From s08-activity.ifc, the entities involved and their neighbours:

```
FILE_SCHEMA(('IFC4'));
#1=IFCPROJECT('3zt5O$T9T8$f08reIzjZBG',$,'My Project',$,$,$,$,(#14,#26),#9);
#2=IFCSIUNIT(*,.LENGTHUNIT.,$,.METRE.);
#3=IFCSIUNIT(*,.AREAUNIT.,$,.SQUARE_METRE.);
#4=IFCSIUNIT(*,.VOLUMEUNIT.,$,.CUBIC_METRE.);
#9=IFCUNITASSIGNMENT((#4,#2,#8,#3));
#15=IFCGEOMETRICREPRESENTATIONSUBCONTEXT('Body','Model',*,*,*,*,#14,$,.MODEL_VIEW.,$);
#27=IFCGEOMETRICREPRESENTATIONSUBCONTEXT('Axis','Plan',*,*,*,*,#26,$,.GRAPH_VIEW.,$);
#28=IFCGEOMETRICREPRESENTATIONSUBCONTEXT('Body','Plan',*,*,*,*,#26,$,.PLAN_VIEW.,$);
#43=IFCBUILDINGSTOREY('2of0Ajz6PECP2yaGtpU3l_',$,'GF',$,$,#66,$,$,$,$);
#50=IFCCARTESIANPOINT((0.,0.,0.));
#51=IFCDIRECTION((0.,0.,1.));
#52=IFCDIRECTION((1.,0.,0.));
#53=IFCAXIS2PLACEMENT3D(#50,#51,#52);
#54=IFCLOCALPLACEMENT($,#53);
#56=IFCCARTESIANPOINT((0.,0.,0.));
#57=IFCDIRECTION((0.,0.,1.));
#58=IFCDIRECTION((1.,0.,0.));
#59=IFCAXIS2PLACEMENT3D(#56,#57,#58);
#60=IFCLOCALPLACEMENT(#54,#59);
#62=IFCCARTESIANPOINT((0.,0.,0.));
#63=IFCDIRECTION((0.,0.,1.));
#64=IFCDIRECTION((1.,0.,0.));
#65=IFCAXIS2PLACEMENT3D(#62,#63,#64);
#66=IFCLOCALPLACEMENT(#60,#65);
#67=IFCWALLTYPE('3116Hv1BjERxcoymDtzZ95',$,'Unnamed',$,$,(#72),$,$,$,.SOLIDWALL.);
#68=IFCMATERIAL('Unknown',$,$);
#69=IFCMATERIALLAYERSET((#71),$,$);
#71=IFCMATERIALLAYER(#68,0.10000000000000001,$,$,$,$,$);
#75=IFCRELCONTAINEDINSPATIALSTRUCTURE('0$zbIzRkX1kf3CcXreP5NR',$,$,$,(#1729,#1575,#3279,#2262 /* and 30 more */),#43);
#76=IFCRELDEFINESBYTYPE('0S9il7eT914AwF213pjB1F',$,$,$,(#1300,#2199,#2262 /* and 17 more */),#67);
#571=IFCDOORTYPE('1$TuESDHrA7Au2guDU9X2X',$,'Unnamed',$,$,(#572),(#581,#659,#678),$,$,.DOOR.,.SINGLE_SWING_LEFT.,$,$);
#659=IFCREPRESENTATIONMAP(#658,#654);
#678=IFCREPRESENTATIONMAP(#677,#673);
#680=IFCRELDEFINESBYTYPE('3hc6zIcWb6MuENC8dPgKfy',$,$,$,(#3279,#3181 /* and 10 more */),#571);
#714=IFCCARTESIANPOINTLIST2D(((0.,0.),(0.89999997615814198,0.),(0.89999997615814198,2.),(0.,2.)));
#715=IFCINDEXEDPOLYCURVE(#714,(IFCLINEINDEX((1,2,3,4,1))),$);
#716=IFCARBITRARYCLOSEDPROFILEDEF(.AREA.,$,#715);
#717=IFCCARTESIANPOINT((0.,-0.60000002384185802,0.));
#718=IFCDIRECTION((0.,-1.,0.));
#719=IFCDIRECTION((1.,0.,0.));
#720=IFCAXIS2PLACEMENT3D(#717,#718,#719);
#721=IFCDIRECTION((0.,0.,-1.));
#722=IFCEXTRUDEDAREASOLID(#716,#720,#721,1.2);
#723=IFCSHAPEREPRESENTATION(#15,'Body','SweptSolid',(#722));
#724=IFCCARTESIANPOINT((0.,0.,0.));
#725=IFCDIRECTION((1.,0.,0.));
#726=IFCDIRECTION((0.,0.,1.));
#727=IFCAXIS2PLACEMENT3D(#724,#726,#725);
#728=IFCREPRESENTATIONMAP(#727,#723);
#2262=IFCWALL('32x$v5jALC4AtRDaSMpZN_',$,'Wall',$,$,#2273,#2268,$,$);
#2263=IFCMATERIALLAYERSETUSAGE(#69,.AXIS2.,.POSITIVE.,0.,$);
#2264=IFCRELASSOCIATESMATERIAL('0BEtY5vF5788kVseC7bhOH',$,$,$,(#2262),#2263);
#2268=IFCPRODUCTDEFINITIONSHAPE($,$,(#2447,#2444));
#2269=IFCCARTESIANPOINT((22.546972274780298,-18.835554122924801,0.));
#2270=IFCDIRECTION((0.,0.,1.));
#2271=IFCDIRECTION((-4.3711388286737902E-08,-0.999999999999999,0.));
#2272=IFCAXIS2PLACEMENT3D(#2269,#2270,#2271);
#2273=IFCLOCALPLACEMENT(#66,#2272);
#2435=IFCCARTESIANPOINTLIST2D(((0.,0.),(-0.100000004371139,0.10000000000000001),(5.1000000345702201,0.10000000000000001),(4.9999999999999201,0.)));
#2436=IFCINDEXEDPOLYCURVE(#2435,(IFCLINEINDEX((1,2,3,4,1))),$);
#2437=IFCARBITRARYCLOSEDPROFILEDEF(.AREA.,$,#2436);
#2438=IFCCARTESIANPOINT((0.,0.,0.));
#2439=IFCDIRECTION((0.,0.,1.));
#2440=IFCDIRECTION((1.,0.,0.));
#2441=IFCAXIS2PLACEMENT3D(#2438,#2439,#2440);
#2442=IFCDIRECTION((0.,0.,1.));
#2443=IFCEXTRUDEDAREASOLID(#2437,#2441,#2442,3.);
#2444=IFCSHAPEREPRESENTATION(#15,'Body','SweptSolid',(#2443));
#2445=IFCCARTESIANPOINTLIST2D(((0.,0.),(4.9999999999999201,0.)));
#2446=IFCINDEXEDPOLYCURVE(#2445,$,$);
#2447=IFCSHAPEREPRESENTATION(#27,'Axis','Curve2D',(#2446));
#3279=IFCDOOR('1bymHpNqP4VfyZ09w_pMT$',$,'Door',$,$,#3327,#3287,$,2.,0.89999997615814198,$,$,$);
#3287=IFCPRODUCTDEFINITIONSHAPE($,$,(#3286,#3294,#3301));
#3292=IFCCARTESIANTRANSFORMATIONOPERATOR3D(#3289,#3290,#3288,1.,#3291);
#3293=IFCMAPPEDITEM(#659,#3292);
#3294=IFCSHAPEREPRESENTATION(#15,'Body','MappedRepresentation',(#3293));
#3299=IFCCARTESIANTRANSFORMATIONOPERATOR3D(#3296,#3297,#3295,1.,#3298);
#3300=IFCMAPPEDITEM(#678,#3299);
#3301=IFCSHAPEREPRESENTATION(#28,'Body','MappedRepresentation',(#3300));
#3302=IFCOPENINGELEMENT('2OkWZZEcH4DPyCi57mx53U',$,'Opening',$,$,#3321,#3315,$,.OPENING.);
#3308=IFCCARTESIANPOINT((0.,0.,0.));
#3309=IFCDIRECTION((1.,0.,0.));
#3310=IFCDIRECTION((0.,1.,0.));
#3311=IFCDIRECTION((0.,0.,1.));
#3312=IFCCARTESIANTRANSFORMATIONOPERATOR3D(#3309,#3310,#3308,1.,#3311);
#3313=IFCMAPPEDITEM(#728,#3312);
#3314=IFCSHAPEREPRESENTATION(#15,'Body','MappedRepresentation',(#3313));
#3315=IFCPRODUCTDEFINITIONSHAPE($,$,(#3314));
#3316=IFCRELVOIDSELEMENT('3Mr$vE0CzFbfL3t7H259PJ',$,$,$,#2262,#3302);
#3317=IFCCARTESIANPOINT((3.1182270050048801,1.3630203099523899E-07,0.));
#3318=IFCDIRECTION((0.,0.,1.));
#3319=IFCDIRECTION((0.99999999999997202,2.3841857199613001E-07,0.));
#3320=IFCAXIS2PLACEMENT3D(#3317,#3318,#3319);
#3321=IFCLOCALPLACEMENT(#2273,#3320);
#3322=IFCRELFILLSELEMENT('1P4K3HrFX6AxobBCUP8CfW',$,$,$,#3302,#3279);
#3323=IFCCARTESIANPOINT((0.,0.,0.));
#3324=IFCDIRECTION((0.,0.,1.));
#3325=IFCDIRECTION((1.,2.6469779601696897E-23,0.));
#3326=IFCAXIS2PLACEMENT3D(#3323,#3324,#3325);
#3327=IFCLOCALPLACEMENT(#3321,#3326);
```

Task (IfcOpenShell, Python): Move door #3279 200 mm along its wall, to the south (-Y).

```python
import ifcopenshell
import ifcopenshell.api.geometry
import ifcopenshell.util.placement
import ifcopenshell.util.unit

model = ifcopenshell.open("s08-activity.ifc")
unit_scale = ifcopenshell.util.unit.calculate_unit_scale(model)

door = model.by_guid("1bymHpNqP4VfyZ09w_pMT$")
opening = door.FillsVoids[0].RelatingOpeningElement
wall = opening.VoidsElements[0].RelatingBuildingElement

wall_matrix = ifcopenshell.util.placement.get_local_placement(wall.ObjectPlacement)
shift = wall_matrix[:3, 0] * 0.2 / unit_scale
before = ifcopenshell.util.placement.get_local_placement(door.ObjectPlacement)[:3, 3].copy()

# The door is placed relative to its opening, so it follows when the opening moves.
matrix = ifcopenshell.util.placement.get_local_placement(opening.ObjectPlacement)
matrix[:3, 3] += shift
ifcopenshell.api.geometry.edit_object_placement(
    model, product=opening, matrix=matrix, is_si=False, should_transform_children=True
)

after = ifcopenshell.util.placement.get_local_placement(door.ObjectPlacement)[:3, 3]
print("door moved by", (after - before).round(3) + 0.0)

model.write("s08-activity_rev.ifc")
```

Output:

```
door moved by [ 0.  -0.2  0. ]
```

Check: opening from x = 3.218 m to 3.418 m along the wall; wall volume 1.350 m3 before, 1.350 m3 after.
